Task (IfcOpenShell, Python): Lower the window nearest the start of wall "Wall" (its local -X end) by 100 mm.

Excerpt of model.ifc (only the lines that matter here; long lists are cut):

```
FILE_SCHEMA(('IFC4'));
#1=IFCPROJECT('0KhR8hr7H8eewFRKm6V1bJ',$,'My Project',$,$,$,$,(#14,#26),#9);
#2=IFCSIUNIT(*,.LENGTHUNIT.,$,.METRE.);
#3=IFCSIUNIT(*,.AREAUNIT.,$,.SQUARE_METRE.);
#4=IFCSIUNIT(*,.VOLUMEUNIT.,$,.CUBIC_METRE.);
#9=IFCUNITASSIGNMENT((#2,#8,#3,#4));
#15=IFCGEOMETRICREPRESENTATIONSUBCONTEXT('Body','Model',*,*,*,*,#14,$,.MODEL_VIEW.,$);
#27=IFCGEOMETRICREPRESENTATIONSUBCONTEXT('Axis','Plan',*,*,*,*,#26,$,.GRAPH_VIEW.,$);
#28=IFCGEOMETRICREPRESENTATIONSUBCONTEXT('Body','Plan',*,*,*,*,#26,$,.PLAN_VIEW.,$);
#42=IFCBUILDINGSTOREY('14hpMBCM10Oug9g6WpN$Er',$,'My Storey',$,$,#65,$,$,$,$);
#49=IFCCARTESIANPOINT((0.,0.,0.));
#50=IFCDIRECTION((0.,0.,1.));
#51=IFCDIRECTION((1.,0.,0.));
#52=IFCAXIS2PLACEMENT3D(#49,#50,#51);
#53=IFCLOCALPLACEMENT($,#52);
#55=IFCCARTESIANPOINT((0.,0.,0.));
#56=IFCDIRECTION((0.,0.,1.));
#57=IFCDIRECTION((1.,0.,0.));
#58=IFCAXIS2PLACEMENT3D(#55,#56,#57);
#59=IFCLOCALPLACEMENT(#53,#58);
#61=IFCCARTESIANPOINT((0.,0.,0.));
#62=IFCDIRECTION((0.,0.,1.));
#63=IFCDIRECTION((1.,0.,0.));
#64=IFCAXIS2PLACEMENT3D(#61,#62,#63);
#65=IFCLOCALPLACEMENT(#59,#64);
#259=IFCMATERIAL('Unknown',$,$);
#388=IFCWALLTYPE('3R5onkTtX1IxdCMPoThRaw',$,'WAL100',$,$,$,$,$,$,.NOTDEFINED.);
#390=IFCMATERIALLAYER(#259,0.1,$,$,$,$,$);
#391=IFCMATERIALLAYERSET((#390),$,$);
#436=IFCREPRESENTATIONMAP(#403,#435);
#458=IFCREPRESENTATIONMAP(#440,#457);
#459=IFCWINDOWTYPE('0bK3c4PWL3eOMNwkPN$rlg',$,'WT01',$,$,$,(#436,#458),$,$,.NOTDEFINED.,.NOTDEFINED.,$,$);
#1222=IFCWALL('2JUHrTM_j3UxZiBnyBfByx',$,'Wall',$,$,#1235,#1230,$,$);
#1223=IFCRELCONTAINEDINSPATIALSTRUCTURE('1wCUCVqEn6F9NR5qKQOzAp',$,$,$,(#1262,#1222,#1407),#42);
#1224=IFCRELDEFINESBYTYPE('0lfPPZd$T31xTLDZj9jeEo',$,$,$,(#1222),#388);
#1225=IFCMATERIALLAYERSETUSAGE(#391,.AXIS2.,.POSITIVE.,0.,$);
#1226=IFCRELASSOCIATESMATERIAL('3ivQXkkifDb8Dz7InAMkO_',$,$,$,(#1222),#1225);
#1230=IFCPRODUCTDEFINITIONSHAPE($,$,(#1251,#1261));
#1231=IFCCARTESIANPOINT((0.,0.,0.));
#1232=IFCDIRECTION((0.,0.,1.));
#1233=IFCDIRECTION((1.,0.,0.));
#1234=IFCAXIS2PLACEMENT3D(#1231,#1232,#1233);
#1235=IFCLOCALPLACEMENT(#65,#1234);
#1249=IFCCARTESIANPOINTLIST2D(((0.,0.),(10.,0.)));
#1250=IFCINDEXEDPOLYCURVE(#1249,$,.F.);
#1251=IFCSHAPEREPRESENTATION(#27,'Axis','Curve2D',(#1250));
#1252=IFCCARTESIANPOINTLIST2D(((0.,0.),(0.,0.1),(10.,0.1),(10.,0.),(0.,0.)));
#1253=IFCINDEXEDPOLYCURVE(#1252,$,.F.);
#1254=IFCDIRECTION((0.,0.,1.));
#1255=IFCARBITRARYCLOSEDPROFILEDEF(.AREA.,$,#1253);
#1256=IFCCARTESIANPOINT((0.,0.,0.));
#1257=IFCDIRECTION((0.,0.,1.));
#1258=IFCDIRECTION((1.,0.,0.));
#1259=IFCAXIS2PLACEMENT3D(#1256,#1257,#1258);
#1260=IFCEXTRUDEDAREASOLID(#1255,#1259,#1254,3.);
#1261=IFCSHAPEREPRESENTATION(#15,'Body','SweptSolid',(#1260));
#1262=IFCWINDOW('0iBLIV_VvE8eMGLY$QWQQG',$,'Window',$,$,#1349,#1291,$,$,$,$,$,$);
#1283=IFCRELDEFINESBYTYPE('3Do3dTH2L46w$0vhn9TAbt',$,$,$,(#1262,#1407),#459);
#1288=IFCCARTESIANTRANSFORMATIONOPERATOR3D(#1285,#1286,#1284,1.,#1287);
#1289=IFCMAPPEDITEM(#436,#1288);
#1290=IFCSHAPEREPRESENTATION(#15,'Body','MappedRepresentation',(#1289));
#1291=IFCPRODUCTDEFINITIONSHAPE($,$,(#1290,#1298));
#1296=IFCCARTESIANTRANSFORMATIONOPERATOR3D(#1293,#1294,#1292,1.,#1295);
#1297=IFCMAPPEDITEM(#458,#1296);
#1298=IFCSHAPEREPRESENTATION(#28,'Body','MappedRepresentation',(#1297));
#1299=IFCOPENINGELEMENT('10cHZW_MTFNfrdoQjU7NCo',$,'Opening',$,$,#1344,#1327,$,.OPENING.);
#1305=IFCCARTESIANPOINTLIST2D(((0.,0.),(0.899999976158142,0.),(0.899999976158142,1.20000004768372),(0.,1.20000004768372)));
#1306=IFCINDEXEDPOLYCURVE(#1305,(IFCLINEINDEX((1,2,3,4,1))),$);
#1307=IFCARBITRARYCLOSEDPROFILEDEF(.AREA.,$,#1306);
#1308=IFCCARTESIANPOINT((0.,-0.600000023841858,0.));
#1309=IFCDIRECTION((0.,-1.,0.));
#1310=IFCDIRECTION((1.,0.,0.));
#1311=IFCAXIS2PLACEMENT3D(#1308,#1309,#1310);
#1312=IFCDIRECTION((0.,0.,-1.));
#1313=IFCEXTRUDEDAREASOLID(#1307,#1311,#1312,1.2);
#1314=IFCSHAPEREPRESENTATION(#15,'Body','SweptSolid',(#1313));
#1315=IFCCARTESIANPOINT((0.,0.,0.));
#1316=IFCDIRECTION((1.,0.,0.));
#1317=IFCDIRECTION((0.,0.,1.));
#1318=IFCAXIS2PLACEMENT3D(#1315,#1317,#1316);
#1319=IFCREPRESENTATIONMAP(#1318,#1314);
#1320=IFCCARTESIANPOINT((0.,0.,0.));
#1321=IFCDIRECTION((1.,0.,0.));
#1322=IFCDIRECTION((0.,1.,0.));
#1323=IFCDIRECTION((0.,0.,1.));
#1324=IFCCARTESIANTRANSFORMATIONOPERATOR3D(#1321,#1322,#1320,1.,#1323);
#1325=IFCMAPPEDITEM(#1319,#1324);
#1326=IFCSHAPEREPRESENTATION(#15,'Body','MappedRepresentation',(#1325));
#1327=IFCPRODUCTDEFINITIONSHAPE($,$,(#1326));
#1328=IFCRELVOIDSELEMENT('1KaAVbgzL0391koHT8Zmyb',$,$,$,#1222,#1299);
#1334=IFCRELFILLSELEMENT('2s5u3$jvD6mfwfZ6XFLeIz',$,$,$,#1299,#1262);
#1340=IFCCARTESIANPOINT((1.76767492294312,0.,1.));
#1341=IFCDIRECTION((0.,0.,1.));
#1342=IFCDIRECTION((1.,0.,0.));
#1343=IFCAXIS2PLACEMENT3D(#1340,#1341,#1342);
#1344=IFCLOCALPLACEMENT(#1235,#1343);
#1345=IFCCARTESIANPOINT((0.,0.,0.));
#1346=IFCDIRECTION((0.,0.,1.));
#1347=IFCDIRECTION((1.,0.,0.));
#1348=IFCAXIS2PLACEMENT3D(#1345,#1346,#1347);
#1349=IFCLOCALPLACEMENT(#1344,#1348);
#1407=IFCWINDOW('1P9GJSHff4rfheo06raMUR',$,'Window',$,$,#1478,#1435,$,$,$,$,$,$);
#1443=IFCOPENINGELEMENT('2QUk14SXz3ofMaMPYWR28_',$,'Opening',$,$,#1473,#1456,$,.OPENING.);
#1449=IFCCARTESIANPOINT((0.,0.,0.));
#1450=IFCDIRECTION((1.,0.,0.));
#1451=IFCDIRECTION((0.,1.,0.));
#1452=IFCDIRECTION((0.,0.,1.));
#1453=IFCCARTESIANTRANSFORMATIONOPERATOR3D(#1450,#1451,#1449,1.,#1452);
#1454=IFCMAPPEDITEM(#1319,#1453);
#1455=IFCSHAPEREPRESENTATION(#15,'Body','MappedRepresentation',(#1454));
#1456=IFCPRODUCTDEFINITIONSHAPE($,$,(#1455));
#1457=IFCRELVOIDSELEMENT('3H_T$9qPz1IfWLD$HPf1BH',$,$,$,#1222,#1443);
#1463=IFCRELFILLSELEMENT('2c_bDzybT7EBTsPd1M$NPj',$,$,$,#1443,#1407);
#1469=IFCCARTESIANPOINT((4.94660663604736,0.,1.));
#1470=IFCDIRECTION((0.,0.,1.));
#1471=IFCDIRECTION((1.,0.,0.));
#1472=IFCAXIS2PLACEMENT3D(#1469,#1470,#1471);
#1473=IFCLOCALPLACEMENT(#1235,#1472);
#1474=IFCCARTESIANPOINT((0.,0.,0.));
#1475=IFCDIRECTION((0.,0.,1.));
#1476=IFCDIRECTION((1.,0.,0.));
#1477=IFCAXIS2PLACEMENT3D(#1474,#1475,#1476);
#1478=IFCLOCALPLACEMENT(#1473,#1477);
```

```python
import numpy as np
import ifcopenshell
import ifcopenshell.api.geometry
import ifcopenshell.util.placement
import ifcopenshell.util.unit

model = ifcopenshell.open("model.ifc")
unit_scale = ifcopenshell.util.unit.calculate_unit_scale(model)

window = model.by_id(1262)
opening = window.FillsVoids[0].RelatingOpeningElement
dz = -0.1 / unit_scale

shift = np.array([0.0, 0.0, dz])
# The window is placed relative to its opening, so it follows when the opening moves.
matrix = ifcopenshell.util.placement.get_local_placement(opening.ObjectPlacement)
matrix[:3, 3] += shift
ifcopenshell.api.geometry.edit_object_placement(
    model, product=opening, matrix=matrix, is_si=False, should_transform_children=True
)

print(f"moved by {dz * unit_scale:+.3f} m")

model.write("model-out.ifc")
```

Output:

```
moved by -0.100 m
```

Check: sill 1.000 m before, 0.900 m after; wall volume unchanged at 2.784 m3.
